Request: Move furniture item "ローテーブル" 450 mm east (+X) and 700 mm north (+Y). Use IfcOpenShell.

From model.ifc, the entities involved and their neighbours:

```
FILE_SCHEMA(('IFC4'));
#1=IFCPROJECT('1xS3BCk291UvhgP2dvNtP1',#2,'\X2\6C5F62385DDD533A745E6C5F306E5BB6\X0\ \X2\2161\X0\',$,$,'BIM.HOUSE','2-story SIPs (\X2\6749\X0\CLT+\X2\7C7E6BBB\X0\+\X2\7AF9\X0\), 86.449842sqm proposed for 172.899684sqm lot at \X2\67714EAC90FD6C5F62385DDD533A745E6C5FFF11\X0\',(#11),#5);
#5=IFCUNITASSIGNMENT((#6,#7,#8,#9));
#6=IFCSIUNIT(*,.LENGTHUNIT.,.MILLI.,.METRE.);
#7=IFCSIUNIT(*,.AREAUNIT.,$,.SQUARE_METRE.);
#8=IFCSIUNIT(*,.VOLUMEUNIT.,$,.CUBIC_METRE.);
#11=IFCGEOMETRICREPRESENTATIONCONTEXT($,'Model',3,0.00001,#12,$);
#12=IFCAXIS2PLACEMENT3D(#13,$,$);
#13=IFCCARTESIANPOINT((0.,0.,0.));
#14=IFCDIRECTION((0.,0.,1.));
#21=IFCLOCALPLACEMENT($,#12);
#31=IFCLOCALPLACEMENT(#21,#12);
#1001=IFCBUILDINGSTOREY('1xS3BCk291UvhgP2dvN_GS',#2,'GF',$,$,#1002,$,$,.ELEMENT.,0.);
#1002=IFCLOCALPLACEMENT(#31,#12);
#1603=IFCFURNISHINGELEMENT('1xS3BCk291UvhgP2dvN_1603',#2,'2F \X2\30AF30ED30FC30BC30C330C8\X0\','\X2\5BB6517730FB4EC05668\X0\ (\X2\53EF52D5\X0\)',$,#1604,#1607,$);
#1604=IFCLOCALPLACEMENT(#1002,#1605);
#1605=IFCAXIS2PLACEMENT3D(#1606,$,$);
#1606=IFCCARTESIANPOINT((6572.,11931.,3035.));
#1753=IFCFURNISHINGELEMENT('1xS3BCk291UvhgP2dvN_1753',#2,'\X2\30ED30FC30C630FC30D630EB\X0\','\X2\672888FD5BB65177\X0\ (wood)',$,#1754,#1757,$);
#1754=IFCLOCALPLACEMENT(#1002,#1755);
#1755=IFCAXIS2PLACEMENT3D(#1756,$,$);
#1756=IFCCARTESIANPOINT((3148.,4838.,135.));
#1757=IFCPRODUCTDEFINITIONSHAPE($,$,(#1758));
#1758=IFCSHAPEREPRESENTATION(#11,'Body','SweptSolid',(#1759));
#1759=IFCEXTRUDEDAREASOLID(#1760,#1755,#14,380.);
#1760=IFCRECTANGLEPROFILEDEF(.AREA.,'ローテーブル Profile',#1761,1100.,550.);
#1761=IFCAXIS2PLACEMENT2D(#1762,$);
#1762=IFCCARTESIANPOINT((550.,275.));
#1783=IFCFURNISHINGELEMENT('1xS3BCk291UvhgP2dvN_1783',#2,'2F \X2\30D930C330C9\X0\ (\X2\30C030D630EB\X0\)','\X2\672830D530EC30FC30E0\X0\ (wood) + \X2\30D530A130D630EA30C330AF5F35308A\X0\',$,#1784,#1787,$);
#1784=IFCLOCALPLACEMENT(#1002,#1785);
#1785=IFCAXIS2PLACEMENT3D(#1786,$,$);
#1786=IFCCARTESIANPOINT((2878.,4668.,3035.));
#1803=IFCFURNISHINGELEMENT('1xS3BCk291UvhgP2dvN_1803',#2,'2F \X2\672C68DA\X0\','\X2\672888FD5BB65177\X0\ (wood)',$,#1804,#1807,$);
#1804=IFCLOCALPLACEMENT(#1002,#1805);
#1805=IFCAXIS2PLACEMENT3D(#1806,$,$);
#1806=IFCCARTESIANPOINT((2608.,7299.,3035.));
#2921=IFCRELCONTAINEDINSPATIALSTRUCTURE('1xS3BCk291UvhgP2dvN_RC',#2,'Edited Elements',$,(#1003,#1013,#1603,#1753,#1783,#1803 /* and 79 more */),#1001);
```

```python
import ifcopenshell
import ifcopenshell.api.geometry
import ifcopenshell.util.placement

model = ifcopenshell.open("model.ifc")

item = model.by_guid("1xS3BCk291UvhgP2dvN_1753")
matrix = ifcopenshell.util.placement.get_local_placement(item.ObjectPlacement)
matrix[0, 3] += 450.0
matrix[1, 3] += 700.0
ifcopenshell.api.geometry.edit_object_placement(model, product=item, matrix=matrix, is_si=False)

print(ifcopenshell.util.placement.get_local_placement(item.ObjectPlacement).round(3) + 0.0)

model.write("model_rev.ifc")
```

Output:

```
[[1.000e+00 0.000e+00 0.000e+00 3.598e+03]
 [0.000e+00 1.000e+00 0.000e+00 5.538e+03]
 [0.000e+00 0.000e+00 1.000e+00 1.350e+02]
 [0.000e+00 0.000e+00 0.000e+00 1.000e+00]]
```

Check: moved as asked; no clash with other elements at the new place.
